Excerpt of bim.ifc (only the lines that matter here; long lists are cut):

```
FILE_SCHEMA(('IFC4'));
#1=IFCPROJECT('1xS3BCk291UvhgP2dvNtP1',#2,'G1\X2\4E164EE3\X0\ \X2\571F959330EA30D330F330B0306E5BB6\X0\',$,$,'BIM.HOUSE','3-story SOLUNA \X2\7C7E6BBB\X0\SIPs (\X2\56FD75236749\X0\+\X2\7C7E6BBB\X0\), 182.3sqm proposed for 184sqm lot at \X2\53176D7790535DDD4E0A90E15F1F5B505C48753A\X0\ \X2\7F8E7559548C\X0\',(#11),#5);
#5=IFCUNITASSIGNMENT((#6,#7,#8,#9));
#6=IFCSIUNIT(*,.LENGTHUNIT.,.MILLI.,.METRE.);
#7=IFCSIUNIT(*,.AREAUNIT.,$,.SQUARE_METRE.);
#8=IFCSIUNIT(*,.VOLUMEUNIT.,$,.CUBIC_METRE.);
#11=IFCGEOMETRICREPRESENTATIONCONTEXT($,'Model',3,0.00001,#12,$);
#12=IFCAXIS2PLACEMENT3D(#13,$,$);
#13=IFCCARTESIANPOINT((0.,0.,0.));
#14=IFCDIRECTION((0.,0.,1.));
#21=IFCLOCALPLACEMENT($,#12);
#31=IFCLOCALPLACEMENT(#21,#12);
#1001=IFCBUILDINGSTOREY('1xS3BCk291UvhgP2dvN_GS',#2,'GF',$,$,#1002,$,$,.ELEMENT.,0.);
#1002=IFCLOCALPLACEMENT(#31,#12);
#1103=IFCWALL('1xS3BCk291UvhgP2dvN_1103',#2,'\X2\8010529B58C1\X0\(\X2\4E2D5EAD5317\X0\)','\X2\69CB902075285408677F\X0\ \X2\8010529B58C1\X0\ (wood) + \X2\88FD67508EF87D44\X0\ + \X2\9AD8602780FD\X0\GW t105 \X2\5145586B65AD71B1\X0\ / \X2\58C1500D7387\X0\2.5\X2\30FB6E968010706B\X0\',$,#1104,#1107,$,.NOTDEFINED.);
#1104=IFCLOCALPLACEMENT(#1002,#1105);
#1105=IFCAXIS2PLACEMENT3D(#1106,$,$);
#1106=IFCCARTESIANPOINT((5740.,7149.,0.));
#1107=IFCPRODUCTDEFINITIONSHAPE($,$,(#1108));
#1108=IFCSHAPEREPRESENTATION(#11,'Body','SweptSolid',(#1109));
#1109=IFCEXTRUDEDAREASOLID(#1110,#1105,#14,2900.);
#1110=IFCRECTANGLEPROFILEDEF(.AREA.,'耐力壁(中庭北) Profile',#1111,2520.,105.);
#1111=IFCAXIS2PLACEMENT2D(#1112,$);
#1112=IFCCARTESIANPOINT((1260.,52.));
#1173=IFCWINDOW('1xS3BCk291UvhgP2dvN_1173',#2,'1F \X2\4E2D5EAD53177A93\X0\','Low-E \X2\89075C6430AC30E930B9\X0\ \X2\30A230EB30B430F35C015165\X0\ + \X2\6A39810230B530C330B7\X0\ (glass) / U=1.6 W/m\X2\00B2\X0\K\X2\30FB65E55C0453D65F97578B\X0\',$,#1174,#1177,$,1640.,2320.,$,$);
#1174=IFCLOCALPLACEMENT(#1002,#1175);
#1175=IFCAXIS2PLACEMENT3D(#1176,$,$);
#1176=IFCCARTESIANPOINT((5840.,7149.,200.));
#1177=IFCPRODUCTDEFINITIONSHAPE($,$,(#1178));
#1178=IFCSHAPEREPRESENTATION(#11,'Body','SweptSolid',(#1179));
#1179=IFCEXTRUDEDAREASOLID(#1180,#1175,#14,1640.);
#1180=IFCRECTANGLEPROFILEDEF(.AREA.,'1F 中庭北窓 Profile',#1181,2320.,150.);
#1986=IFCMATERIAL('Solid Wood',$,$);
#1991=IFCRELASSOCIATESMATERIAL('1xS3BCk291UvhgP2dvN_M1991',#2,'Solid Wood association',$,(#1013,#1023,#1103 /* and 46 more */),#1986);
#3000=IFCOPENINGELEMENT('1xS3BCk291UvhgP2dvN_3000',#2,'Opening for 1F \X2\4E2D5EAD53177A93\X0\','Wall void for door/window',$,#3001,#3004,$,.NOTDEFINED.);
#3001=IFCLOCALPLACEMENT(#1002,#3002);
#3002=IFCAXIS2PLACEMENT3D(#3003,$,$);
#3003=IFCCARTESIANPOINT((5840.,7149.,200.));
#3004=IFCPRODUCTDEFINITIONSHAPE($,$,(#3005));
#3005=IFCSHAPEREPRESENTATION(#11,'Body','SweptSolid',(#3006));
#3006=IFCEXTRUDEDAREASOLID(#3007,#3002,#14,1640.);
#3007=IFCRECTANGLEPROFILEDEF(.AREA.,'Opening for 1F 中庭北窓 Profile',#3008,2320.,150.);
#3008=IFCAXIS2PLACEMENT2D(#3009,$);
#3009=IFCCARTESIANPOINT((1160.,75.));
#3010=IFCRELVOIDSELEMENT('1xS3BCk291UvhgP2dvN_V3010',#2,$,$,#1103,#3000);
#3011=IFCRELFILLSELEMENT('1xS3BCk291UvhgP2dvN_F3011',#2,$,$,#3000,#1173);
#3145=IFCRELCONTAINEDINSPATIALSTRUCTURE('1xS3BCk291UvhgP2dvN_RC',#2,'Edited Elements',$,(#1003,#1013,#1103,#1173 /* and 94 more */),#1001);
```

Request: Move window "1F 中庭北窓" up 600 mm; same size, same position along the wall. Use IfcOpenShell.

```python
import numpy as np
import ifcopenshell
import ifcopenshell.api.geometry
import ifcopenshell.util.placement
import ifcopenshell.util.unit

model = ifcopenshell.open("bim.ifc")
unit_scale = ifcopenshell.util.unit.calculate_unit_scale(model)

window = model.by_id(1173)
opening = window.FillsVoids[0].RelatingOpeningElement
dz = 0.6 / unit_scale

shift = np.array([0.0, 0.0, dz])
# The window is not placed relative to its opening, so move both.
for product in (opening, window):
    matrix = ifcopenshell.util.placement.get_local_placement(product.ObjectPlacement)
    matrix[:3, 3] += shift
    ifcopenshell.api.geometry.edit_object_placement(model, product=product, matrix=matrix, is_si=False)

print(f"moved by {dz * unit_scale:+.3f} m")

model.write("bim-out.ifc")
```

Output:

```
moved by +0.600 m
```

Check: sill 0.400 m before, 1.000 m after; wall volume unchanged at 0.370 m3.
